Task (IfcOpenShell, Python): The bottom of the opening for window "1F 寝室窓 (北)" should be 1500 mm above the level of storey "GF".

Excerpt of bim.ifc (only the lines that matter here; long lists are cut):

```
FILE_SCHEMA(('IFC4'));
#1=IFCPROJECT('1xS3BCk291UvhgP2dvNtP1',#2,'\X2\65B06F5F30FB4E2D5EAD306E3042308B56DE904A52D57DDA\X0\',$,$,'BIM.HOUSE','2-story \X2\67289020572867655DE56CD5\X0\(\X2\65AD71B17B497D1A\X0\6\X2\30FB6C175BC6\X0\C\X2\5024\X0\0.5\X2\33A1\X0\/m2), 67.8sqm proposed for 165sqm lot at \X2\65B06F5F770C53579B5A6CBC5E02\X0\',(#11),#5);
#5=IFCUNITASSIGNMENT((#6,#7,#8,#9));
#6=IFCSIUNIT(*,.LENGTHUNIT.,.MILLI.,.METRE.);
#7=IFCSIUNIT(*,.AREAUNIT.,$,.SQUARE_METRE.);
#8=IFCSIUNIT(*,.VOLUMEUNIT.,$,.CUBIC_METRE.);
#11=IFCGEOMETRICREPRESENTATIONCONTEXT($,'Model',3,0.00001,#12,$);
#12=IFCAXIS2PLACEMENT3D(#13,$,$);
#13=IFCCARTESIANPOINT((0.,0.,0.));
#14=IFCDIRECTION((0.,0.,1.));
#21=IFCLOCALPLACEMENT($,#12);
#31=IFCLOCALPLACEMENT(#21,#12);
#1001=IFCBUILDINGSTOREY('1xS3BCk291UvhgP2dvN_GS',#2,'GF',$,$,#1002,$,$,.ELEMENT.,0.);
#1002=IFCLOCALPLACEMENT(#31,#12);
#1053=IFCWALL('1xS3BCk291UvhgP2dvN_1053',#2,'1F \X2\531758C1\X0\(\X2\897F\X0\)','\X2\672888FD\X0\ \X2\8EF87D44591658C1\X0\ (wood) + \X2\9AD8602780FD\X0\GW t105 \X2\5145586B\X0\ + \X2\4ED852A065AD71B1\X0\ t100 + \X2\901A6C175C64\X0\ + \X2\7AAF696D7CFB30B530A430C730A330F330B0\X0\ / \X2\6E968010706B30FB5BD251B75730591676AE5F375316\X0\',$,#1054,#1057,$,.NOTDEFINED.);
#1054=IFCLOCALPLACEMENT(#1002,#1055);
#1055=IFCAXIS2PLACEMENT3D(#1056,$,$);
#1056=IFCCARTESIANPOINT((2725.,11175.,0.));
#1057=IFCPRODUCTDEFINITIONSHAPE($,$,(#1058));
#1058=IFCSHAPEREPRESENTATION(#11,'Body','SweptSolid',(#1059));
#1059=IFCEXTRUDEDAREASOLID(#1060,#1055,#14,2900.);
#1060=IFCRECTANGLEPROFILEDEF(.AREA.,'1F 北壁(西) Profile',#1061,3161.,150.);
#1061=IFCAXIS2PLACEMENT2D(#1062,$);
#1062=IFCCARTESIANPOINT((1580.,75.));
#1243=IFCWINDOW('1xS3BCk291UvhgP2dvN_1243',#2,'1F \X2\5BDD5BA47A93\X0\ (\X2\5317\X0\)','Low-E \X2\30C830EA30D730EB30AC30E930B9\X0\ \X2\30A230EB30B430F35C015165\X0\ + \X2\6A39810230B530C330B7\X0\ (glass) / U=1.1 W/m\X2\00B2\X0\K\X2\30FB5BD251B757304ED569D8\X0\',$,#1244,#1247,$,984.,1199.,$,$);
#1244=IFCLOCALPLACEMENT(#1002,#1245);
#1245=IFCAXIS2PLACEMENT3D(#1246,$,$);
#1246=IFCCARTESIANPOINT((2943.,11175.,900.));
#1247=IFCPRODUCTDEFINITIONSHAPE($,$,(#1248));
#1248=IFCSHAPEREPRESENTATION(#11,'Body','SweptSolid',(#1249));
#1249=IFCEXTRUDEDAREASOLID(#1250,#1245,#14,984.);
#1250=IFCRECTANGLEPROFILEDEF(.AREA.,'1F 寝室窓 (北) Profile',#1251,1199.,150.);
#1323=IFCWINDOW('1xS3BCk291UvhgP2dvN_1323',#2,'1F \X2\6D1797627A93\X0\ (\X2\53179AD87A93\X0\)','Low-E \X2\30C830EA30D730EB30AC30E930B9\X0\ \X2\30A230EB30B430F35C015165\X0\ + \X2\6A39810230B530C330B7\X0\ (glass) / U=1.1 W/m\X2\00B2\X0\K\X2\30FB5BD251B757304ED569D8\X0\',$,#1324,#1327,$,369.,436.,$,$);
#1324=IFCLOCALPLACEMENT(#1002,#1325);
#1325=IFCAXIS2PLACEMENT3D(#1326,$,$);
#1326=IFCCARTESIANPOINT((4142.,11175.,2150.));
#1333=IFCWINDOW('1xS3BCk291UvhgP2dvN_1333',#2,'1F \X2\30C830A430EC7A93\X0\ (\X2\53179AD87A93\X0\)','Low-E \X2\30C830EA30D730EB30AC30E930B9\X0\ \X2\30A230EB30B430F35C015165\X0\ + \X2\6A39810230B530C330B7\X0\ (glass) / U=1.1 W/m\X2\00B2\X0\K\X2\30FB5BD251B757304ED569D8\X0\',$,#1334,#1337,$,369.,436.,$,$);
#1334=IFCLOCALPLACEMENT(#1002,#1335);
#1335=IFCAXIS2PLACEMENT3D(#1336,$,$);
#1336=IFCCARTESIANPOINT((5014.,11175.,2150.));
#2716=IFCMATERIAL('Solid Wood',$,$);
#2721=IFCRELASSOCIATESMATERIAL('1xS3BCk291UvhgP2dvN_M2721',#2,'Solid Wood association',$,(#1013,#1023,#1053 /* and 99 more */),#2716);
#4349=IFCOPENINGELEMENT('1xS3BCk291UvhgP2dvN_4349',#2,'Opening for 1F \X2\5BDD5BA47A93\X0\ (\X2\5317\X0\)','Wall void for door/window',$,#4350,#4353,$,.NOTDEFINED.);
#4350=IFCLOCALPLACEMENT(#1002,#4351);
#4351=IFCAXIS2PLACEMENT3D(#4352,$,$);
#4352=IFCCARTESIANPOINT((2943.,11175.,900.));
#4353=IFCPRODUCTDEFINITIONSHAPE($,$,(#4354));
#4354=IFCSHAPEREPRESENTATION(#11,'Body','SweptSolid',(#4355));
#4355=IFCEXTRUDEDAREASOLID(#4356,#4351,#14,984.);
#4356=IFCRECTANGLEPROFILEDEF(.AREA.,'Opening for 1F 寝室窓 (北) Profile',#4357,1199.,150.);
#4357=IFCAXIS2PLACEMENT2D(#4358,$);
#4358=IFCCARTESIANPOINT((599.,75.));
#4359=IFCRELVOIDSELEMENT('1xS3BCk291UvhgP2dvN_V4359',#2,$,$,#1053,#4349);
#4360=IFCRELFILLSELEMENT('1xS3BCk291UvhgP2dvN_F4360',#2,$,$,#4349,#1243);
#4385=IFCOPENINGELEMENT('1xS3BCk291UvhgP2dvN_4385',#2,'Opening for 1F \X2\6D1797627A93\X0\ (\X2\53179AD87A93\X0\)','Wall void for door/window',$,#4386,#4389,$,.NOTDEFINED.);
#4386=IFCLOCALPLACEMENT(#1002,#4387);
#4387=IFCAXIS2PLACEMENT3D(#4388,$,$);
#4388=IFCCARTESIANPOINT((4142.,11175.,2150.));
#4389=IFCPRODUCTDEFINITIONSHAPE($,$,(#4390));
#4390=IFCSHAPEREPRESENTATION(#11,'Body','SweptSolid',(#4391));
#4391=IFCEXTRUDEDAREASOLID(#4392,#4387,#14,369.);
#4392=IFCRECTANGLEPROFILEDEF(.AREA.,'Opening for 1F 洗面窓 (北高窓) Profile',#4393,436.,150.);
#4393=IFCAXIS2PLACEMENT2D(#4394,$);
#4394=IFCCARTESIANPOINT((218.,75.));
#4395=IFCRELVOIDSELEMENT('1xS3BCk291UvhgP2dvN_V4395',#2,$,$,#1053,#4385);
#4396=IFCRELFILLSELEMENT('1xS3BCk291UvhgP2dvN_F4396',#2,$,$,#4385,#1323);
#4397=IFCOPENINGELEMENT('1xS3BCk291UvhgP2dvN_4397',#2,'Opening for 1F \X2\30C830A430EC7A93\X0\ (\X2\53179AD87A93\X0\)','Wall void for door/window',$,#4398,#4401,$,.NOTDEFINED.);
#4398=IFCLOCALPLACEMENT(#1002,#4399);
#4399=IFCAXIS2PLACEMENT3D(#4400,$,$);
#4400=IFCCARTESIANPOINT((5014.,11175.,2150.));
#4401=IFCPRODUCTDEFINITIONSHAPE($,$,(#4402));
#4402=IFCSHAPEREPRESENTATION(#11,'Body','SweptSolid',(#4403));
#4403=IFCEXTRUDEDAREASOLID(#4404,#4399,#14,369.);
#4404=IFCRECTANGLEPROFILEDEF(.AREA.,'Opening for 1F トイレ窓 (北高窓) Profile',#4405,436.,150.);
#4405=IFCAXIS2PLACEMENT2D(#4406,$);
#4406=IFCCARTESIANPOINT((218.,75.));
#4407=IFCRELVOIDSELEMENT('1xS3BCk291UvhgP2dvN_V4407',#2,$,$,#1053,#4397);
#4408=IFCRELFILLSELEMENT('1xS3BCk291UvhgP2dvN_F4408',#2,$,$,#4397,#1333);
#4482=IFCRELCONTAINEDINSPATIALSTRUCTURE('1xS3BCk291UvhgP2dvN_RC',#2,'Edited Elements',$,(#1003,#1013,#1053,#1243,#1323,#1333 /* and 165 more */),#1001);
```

```python
import numpy as np
import ifcopenshell
import ifcopenshell.api.geometry
import ifcopenshell.geom
import ifcopenshell.util.element
import ifcopenshell.util.placement
import ifcopenshell.util.shape
import ifcopenshell.util.unit

model = ifcopenshell.open("bim.ifc")
unit_scale = ifcopenshell.util.unit.calculate_unit_scale(model)

window = model.by_id(1243)
opening = window.FillsVoids[0].RelatingOpeningElement
storey = ifcopenshell.util.element.get_container(window, ifc_class="IfcBuildingStorey")
level = ifcopenshell.util.placement.get_local_placement(storey.ObjectPlacement)[2, 3]

# The opening's origin need not be at the sill, so measure its lowest point.
shape = ifcopenshell.geom.create_shape(ifcopenshell.geom.settings(), opening)
bottom = ifcopenshell.util.shape.get_shape_bottom_elevation(shape, shape.geometry) / unit_scale
dz = level + 1.5 / unit_scale - bottom

shift = np.array([0.0, 0.0, dz])
# The window is not placed relative to its opening, so move both.
for product in (opening, window):
    matrix = ifcopenshell.util.placement.get_local_placement(product.ObjectPlacement)
    matrix[:3, 3] += shift
    ifcopenshell.api.geometry.edit_object_placement(model, product=product, matrix=matrix, is_si=False)

print(f"moved by {dz * unit_scale:+.3f} m")

model.write("bim_edited.ifc")
```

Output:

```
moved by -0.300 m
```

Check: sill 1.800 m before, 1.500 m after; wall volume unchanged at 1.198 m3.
